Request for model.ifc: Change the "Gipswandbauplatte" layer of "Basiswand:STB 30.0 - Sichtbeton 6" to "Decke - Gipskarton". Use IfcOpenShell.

First a look at what the model holds.

```python
import ifcopenshell
import ifcopenshell.util.element

model = ifcopenshell.open("model.ifc")
print(model.schema)
for layer_set in model.by_type("IfcMaterialLayerSet"):
    if layer_set.LayerSetName == "Basiswand:STB 30.0 - Sichtbeton 6":
        for layer in layer_set.MaterialLayers:
            print(layer.id(), layer.Material and layer.Material.Name, layer.LayerThickness, sep=" | ")
        print(len(ifcopenshell.util.element.get_elements_by_material(model, layer_set)), "elements and types use it")
print(sorted(m.Name for m in model.by_type("IfcMaterial") if m.Name)[:60])
```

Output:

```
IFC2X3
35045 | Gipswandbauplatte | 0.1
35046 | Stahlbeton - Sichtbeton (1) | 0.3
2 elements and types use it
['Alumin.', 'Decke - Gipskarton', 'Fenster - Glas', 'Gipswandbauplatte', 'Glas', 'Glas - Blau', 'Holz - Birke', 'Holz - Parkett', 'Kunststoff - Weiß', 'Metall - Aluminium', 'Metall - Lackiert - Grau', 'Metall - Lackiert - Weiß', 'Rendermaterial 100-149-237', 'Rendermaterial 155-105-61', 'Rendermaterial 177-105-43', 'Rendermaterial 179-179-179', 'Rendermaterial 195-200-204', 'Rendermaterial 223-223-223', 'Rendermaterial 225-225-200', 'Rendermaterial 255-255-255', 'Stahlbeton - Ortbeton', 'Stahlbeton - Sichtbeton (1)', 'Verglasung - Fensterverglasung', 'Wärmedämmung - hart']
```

```python
import ifcopenshell
import ifcopenshell.api.material

model = ifcopenshell.open("model.ifc")

layer_set = next(s for s in model.by_type("IfcMaterialLayerSet") if s.LayerSetName == "Basiswand:STB 30.0 - Sichtbeton 6")
layer = next(l for l in layer_set.MaterialLayers if l.Material and l.Material.Name == "Gipswandbauplatte")
material = next(m for m in model.by_type("IfcMaterial") if m.Name == "Decke - Gipskarton")

# Point this one layer at the other material; renaming the old one would change it everywhere.
ifcopenshell.api.material.edit_layer(model, layer=layer, attributes={}, material=material)

print([l.Material.Name if l.Material else None for l in layer_set.MaterialLayers])

model.write("model_edited.ifc")
```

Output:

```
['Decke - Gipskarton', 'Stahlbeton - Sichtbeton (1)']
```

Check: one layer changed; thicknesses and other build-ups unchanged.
